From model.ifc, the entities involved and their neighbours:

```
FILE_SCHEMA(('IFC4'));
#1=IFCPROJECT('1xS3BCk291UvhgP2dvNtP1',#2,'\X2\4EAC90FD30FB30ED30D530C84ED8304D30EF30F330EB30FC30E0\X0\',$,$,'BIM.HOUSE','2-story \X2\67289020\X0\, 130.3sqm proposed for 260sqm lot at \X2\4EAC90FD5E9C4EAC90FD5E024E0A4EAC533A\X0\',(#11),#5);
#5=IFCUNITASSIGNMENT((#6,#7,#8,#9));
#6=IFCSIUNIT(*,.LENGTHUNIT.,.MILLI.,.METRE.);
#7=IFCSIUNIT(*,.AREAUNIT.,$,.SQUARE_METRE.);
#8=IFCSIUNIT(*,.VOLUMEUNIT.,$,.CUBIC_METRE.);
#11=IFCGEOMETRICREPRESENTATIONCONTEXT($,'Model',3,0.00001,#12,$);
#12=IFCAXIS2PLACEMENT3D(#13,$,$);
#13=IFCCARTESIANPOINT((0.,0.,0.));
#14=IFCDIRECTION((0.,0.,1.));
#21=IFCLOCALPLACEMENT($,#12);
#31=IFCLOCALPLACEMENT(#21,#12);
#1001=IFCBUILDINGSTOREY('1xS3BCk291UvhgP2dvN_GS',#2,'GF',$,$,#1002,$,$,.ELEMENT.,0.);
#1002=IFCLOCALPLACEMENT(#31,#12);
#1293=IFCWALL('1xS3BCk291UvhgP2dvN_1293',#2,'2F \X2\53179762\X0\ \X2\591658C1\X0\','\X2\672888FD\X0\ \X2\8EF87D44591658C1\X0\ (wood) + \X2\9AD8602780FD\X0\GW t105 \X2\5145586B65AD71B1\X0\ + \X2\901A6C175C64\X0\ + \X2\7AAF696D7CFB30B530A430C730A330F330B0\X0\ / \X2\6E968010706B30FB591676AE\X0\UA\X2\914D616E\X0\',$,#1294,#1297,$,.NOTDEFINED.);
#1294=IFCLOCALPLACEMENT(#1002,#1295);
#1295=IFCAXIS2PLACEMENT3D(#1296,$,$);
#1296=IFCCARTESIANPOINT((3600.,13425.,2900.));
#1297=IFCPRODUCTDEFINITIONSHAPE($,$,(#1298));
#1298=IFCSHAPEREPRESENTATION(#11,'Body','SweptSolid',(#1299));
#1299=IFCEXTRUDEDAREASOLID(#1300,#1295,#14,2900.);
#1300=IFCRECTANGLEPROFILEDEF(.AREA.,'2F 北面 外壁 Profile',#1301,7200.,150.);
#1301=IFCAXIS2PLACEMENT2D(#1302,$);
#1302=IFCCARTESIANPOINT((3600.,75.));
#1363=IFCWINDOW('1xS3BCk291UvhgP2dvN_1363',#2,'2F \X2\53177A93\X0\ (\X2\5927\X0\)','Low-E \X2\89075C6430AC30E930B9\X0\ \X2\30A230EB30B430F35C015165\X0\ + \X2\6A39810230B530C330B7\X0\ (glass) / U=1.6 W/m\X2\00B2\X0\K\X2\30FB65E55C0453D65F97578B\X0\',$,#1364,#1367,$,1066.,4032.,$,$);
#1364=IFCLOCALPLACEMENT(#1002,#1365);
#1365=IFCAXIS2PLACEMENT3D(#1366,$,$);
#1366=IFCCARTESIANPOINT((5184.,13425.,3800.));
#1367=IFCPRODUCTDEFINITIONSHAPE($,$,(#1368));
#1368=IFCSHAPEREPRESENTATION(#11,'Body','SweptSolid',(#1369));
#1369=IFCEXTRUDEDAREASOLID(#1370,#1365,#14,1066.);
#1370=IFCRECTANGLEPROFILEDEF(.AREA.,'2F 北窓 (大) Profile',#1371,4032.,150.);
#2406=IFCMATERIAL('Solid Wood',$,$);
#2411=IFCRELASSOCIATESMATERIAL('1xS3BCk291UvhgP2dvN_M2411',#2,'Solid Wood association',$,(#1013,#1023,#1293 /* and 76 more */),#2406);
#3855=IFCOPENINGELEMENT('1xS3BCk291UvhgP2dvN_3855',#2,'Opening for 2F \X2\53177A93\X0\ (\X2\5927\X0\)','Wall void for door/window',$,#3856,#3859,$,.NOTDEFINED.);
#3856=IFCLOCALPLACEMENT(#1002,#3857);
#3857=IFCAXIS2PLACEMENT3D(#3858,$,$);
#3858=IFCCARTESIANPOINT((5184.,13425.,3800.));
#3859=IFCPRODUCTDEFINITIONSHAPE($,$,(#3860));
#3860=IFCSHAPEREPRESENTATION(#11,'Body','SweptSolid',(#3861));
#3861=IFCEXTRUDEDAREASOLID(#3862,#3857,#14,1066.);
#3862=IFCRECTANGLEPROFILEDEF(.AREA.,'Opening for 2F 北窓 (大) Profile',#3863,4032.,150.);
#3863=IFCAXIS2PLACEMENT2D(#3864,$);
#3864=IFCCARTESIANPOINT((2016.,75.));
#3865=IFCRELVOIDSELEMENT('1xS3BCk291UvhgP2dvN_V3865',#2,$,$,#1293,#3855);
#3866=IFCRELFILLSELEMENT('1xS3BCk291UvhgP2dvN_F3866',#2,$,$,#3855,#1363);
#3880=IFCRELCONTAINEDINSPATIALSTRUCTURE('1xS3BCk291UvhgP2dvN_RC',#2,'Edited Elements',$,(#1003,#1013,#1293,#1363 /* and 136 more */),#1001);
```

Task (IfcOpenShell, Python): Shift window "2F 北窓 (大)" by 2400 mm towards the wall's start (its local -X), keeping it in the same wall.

```python
import ifcopenshell
import ifcopenshell.api.geometry
import ifcopenshell.util.placement
import ifcopenshell.util.unit

model = ifcopenshell.open("model.ifc")
unit_scale = ifcopenshell.util.unit.calculate_unit_scale(model)

window = model.by_guid("1xS3BCk291UvhgP2dvN_1363")
opening = window.FillsVoids[0].RelatingOpeningElement
wall = opening.VoidsElements[0].RelatingBuildingElement

wall_matrix = ifcopenshell.util.placement.get_local_placement(wall.ObjectPlacement)
shift = wall_matrix[:3, 0] * -2.4 / unit_scale
before = ifcopenshell.util.placement.get_local_placement(window.ObjectPlacement)[:3, 3].copy()

# The window is not placed relative to its opening, so move both.
for product in (opening, window):
    matrix = ifcopenshell.util.placement.get_local_placement(product.ObjectPlacement)
    matrix[:3, 3] += shift
    ifcopenshell.api.geometry.edit_object_placement(model, product=product, matrix=matrix, is_si=False)

after = ifcopenshell.util.placement.get_local_placement(window.ObjectPlacement)[:3, 3]
print("window moved by", (after - before).round(3) + 0.0)

model.write("model_v2.ifc")
```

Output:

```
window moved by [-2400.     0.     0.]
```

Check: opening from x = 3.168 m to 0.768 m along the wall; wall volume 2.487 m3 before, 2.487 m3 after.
